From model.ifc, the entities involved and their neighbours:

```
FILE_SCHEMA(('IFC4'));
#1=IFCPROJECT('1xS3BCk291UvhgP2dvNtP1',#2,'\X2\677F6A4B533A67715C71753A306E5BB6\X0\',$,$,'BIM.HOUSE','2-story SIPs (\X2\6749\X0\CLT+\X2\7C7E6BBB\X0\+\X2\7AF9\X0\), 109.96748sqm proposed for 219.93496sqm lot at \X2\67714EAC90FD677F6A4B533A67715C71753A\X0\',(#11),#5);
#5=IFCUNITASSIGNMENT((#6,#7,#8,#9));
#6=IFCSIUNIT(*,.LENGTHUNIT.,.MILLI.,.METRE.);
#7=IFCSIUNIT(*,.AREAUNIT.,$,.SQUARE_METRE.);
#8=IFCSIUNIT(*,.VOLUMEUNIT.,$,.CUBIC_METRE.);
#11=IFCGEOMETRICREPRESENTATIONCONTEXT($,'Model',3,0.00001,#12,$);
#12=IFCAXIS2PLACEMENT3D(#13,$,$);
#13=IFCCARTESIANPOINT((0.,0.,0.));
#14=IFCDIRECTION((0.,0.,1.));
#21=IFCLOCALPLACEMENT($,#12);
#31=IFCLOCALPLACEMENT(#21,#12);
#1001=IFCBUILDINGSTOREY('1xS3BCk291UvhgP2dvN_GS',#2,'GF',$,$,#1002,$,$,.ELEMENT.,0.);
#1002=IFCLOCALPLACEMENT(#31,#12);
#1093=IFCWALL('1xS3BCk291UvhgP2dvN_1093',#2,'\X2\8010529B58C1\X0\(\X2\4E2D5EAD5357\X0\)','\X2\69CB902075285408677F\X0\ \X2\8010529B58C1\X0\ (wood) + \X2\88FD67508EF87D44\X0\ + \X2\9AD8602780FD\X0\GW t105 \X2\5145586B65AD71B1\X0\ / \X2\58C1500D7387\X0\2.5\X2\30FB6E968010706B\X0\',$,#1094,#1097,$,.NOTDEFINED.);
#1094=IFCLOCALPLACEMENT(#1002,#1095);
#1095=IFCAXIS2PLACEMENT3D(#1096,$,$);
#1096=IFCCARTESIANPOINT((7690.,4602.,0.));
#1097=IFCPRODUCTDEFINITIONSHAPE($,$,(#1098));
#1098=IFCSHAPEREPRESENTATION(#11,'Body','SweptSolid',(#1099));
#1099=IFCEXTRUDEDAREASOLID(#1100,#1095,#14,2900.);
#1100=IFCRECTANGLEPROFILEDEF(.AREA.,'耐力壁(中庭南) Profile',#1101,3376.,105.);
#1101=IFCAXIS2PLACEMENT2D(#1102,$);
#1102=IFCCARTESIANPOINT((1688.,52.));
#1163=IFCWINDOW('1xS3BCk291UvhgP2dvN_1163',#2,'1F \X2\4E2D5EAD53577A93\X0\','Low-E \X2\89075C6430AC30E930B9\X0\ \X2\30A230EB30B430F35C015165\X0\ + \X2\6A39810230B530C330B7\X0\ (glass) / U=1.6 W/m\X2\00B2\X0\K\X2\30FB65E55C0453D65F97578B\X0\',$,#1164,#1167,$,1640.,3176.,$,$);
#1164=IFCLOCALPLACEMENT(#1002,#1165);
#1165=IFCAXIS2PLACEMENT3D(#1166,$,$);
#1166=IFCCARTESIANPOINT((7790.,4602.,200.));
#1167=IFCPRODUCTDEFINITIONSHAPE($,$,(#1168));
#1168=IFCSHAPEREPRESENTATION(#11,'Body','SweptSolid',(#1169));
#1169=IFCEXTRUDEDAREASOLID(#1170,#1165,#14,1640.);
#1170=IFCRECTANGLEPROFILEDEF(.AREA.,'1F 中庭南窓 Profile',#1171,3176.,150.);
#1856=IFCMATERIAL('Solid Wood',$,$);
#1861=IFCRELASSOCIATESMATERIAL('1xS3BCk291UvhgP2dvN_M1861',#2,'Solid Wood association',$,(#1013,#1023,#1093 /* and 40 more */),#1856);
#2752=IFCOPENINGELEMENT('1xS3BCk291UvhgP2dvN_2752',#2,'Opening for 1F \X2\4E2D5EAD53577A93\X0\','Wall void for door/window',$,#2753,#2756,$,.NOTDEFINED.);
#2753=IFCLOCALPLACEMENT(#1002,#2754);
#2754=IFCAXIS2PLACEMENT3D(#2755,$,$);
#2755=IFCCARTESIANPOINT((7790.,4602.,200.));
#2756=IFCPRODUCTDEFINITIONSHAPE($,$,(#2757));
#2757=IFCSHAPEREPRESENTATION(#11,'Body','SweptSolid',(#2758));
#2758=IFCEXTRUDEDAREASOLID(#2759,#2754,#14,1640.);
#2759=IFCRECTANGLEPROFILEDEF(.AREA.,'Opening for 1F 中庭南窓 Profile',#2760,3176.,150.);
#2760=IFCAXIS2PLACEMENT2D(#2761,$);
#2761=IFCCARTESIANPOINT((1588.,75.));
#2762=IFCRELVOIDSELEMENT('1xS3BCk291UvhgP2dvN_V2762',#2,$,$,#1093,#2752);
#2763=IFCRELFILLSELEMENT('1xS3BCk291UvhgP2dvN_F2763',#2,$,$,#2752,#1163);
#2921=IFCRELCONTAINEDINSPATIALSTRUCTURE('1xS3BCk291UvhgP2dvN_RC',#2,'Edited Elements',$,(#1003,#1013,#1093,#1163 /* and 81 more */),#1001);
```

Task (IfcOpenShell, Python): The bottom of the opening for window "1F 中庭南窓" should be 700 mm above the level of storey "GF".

```python
import numpy as np
import ifcopenshell
import ifcopenshell.api.geometry
import ifcopenshell.geom
import ifcopenshell.util.element
import ifcopenshell.util.placement
import ifcopenshell.util.shape
import ifcopenshell.util.unit

model = ifcopenshell.open("model.ifc")
unit_scale = ifcopenshell.util.unit.calculate_unit_scale(model)

window = model.by_guid("1xS3BCk291UvhgP2dvN_1163")
opening = window.FillsVoids[0].RelatingOpeningElement
storey = ifcopenshell.util.element.get_container(window, ifc_class="IfcBuildingStorey")
level = ifcopenshell.util.placement.get_local_placement(storey.ObjectPlacement)[2, 3]

# The opening's origin need not be at the sill, so measure its lowest point.
shape = ifcopenshell.geom.create_shape(ifcopenshell.geom.settings(), opening)
bottom = ifcopenshell.util.shape.get_shape_bottom_elevation(shape, shape.geometry) / unit_scale
dz = level + 0.7 / unit_scale - bottom

shift = np.array([0.0, 0.0, dz])
# The window is not placed relative to its opening, so move both.
for product in (opening, window):
    matrix = ifcopenshell.util.placement.get_local_placement(product.ObjectPlacement)
    matrix[:3, 3] += shift
    ifcopenshell.api.geometry.edit_object_placement(model, product=product, matrix=matrix, is_si=False)

print(f"moved by {dz * unit_scale:+.3f} m")

model.write("model_edited.ifc")
```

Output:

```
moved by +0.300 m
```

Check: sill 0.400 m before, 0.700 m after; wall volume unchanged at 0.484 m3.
